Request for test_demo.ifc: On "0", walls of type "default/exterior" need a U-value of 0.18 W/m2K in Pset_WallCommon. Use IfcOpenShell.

First a look at what the model holds.

```python
import ifcopenshell
import ifcopenshell.util.element

model = ifcopenshell.open("test_demo.ifc")
print(model.schema)
storey = next(s for s in model.by_type("IfcBuildingStorey") if s.Name == "0")
walls = [e for e in ifcopenshell.util.element.get_decomposition(storey) if e.is_a("IfcWall")]
seen = {}
for e in walls:
    element_type = ifcopenshell.util.element.get_type(e)
    key = (element_type.Name if element_type != e and element_type else None, ifcopenshell.util.element.get_pset(e, "Pset_WallCommon", "ThermalTransmittance"))
    seen[key] = seen.get(key, 0) + 1
for (name, value), count in sorted(seen.items(), key=str):
    print(count, "x", name, "|", value)
```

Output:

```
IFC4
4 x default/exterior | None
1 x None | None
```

```python
import ifcopenshell
import ifcopenshell.api.pset
import ifcopenshell.util.element

model = ifcopenshell.open("test_demo.ifc")

storey = next(s for s in model.by_type("IfcBuildingStorey") if s.Name == "0")
walls = [e for e in ifcopenshell.util.element.get_decomposition(storey) if e.is_a("IfcWall")]

count = 0
for e in walls:
    element_type = ifcopenshell.util.element.get_type(e)
    if element_type in (None, e) or element_type.Name != "default/exterior":
        continue
    # add_pset returns the element's existing set when there is one.
    pset = ifcopenshell.api.pset.add_pset(model, product=e, name="Pset_WallCommon")
    ifcopenshell.api.pset.edit_pset(model, pset=pset, properties={"ThermalTransmittance": 0.18})
    count += 1

print(count, "walls updated")

model.write("test_demo_edited.ifc")
```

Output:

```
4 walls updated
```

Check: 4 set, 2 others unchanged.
